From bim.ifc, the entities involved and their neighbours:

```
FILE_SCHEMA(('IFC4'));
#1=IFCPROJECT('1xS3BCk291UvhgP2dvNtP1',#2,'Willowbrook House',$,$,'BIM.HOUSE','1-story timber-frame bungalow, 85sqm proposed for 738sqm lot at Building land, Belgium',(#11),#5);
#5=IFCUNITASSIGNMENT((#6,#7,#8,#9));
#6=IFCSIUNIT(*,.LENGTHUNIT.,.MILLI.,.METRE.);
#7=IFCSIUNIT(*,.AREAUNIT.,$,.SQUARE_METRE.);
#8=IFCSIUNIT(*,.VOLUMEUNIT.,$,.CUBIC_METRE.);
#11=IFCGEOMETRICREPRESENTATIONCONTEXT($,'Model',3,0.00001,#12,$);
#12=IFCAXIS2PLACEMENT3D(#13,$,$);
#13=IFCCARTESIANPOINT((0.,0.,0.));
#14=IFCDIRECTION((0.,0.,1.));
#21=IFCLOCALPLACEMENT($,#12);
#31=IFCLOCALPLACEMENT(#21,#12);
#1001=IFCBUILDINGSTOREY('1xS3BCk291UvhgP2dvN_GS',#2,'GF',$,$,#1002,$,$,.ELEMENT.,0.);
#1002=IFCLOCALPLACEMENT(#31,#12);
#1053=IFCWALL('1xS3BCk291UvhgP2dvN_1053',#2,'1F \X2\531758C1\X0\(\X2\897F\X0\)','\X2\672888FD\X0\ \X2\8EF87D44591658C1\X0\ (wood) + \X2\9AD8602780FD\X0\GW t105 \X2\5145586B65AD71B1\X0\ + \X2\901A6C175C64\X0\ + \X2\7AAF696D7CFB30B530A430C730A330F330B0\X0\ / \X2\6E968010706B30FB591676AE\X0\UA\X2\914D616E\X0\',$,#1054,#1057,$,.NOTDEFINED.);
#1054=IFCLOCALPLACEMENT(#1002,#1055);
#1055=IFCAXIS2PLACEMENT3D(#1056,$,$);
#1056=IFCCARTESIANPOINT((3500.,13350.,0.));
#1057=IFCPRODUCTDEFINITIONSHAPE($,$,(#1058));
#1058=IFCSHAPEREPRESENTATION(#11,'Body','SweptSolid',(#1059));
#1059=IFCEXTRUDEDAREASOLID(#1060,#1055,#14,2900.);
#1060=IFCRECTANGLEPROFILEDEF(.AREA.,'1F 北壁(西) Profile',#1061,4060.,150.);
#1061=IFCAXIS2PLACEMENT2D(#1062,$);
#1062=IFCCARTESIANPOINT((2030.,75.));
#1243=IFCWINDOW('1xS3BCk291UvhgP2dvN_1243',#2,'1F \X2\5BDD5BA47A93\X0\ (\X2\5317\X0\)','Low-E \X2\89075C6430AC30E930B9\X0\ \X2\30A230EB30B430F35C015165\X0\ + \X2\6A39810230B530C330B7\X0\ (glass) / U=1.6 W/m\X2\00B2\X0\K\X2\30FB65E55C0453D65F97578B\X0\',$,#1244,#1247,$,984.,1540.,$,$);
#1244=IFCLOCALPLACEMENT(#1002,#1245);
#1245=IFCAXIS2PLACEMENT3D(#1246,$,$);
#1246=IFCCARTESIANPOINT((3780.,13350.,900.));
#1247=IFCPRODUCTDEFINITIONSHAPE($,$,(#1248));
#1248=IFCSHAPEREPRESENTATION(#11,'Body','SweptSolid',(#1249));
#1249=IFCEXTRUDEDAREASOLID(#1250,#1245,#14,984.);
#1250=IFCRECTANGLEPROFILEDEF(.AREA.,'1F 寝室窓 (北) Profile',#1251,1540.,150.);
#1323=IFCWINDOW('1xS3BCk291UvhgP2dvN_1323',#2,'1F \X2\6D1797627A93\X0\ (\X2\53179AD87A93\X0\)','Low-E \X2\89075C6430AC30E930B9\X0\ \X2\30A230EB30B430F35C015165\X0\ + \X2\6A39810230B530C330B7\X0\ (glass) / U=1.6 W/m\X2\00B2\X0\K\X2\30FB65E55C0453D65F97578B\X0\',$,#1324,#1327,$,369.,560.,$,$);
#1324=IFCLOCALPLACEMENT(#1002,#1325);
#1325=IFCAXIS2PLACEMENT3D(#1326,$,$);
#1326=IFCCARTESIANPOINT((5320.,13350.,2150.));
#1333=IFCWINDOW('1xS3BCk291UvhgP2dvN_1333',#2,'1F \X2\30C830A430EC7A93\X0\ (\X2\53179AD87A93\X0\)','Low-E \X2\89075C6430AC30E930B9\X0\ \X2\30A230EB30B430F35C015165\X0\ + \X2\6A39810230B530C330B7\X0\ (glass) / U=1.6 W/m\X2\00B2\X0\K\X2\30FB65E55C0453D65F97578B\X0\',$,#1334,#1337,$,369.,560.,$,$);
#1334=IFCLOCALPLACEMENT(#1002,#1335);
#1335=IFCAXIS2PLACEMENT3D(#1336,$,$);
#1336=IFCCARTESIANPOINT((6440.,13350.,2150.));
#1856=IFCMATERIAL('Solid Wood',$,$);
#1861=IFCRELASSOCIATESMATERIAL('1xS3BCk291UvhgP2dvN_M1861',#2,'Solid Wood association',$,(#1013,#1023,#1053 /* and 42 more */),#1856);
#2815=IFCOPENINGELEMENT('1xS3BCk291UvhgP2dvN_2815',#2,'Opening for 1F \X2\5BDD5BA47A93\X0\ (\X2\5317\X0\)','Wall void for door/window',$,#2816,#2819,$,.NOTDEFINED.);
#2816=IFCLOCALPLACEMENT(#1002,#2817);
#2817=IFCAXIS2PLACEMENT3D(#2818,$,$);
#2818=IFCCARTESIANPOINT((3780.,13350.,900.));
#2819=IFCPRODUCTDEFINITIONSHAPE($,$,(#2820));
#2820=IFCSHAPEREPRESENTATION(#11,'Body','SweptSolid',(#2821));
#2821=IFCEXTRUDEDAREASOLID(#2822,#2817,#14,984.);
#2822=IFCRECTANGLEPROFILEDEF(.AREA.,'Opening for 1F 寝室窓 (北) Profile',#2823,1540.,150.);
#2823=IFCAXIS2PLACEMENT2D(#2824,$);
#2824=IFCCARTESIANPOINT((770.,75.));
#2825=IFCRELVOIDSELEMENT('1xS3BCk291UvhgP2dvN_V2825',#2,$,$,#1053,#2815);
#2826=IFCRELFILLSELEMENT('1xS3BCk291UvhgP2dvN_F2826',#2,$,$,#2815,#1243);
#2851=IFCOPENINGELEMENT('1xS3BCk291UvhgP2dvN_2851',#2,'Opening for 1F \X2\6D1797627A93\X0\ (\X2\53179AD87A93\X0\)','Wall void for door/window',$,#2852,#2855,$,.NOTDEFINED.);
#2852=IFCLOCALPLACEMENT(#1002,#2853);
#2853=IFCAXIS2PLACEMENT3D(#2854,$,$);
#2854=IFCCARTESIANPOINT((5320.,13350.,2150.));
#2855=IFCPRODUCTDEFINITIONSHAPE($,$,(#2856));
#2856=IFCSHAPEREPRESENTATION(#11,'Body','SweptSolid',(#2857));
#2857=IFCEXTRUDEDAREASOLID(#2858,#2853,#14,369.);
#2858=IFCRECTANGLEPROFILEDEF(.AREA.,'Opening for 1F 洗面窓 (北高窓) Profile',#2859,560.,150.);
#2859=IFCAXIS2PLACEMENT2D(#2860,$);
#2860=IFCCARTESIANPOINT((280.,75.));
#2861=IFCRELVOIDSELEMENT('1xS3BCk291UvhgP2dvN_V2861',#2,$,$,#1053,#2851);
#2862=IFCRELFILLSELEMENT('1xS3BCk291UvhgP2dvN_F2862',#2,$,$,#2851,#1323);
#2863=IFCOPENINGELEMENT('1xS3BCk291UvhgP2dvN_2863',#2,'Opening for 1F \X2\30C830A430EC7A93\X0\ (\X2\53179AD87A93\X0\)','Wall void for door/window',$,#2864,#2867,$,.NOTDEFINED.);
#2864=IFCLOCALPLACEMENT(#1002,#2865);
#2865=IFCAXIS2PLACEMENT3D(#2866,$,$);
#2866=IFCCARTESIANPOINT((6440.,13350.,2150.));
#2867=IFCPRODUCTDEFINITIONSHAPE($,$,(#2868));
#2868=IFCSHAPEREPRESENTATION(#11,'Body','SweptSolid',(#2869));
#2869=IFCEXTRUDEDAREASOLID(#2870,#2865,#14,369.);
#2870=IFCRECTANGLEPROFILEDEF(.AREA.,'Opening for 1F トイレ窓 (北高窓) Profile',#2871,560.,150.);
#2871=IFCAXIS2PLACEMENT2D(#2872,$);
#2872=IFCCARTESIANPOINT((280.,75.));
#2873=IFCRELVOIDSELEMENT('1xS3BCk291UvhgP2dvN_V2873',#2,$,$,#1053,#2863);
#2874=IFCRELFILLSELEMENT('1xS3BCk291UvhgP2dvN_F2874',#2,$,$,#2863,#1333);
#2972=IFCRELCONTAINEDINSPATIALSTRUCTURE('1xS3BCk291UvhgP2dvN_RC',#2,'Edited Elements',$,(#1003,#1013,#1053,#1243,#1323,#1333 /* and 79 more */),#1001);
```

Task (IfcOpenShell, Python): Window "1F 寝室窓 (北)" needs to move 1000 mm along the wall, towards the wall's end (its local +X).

```python
import ifcopenshell
import ifcopenshell.api.geometry
import ifcopenshell.util.placement

model = ifcopenshell.open("bim.ifc")

window = model.by_guid("1xS3BCk291UvhgP2dvN_1243")
opening = window.FillsVoids[0].RelatingOpeningElement
wall = opening.VoidsElements[0].RelatingBuildingElement

wall_matrix = ifcopenshell.util.placement.get_local_placement(wall.ObjectPlacement)
shift = wall_matrix[:3, 0] * 1000.0
before = ifcopenshell.util.placement.get_local_placement(window.ObjectPlacement)[:3, 3].copy()

# The window is not placed relative to its opening, so move both.
for product in (opening, window):
    matrix = ifcopenshell.util.placement.get_local_placement(product.ObjectPlacement)
    matrix[:3, 3] += shift
    ifcopenshell.api.geometry.edit_object_placement(model, product=product, matrix=matrix, is_si=False)

after = ifcopenshell.util.placement.get_local_placement(window.ObjectPlacement)[:3, 3]
print("window moved by", (after - before).round(3) + 0.0)

model.write("bim_v2.ifc")
```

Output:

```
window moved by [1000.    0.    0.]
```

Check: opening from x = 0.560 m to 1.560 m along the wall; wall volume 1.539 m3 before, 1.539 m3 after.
